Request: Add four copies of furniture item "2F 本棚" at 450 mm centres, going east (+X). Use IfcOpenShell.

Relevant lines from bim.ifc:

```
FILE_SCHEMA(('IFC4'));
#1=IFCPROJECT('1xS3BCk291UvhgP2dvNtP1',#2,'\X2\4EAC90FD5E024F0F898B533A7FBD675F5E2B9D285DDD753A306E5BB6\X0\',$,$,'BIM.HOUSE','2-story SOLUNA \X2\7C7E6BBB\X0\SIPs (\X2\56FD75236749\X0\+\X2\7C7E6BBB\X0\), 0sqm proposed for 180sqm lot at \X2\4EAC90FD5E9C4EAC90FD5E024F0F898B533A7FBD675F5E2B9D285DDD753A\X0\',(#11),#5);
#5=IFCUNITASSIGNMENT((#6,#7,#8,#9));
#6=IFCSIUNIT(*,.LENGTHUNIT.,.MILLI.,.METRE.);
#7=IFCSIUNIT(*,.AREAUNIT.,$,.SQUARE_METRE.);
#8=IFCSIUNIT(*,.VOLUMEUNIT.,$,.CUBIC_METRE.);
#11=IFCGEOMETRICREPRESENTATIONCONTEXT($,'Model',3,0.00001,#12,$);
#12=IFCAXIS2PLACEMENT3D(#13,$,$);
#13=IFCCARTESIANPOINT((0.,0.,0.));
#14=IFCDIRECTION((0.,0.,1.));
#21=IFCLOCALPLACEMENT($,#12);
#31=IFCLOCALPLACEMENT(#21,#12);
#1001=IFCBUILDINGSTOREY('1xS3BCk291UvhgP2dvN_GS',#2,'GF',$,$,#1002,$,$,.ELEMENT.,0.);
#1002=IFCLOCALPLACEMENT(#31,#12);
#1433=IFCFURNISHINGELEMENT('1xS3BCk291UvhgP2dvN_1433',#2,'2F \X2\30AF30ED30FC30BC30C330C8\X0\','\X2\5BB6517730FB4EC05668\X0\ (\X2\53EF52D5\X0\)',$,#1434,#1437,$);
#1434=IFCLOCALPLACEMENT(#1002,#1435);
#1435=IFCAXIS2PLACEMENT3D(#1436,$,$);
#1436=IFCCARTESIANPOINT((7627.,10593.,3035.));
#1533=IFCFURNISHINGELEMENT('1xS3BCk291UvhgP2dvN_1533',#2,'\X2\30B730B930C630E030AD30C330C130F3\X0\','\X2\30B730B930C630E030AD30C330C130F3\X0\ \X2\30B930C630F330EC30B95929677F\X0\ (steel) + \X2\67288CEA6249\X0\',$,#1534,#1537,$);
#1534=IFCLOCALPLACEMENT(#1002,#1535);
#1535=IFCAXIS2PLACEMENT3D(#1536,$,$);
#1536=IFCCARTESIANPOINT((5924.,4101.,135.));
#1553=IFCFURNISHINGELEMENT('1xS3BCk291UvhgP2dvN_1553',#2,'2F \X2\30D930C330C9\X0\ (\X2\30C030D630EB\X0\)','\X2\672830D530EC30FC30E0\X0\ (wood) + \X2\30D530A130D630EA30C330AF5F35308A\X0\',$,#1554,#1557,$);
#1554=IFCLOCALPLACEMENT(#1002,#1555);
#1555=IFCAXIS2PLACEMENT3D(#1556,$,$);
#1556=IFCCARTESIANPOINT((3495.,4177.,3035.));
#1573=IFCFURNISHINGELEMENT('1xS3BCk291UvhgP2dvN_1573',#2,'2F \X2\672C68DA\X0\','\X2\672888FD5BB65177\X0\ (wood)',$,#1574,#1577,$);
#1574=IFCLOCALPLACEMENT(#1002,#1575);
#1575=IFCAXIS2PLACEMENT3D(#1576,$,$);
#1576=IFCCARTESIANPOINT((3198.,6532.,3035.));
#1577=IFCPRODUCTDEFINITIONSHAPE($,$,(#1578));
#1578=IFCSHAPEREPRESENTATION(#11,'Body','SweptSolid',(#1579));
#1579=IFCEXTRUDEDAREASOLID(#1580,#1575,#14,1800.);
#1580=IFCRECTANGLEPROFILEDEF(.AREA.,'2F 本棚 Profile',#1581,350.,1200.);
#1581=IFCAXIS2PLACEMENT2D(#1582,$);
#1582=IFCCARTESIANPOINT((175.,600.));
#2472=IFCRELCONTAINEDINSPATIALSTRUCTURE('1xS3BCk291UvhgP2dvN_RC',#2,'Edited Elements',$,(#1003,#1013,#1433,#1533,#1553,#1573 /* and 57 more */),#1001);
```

```python
import numpy as np
import ifcopenshell
import ifcopenshell.api.geometry
import ifcopenshell.api.root
import ifcopenshell.util.element
import ifcopenshell.util.placement

model = ifcopenshell.open("bim.ifc")


def reuse_history(source, copy):
    """copy_class also copies each property set's owner history, people and application; keep the originals."""
    for rel in copy.IsDefinedBy:
        if rel.is_a("IfcRelDefinesByProperties") and (history := rel.RelatingPropertyDefinition.OwnerHistory):
            rel.RelatingPropertyDefinition.OwnerHistory = source.OwnerHistory
            ifcopenshell.util.element.remove_deep2(model, history)


source = model.by_id(1573)
base = ifcopenshell.util.placement.get_local_placement(source.ObjectPlacement)
step = np.array([1.0, 0.0, 0.0]) * 450.0

for i in range(1, 5):
    copy = ifcopenshell.api.root.copy_class(model, product=source)
    copy.Representation = ifcopenshell.util.element.copy_deep(
        model, source.Representation, exclude=["IfcGeometricRepresentationContext", "IfcRepresentationMap"]
    )
    reuse_history(source, copy)
    matrix = base.copy()
    matrix[:3, 3] += i * step
    print("added at", matrix[:3, 3].round(3) + 0.0)
    ifcopenshell.api.geometry.edit_object_placement(model, product=copy, matrix=matrix, is_si=False)

model.write("bim-out.ifc")
```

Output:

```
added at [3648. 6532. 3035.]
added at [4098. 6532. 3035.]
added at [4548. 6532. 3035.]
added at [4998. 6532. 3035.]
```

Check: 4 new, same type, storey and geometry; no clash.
